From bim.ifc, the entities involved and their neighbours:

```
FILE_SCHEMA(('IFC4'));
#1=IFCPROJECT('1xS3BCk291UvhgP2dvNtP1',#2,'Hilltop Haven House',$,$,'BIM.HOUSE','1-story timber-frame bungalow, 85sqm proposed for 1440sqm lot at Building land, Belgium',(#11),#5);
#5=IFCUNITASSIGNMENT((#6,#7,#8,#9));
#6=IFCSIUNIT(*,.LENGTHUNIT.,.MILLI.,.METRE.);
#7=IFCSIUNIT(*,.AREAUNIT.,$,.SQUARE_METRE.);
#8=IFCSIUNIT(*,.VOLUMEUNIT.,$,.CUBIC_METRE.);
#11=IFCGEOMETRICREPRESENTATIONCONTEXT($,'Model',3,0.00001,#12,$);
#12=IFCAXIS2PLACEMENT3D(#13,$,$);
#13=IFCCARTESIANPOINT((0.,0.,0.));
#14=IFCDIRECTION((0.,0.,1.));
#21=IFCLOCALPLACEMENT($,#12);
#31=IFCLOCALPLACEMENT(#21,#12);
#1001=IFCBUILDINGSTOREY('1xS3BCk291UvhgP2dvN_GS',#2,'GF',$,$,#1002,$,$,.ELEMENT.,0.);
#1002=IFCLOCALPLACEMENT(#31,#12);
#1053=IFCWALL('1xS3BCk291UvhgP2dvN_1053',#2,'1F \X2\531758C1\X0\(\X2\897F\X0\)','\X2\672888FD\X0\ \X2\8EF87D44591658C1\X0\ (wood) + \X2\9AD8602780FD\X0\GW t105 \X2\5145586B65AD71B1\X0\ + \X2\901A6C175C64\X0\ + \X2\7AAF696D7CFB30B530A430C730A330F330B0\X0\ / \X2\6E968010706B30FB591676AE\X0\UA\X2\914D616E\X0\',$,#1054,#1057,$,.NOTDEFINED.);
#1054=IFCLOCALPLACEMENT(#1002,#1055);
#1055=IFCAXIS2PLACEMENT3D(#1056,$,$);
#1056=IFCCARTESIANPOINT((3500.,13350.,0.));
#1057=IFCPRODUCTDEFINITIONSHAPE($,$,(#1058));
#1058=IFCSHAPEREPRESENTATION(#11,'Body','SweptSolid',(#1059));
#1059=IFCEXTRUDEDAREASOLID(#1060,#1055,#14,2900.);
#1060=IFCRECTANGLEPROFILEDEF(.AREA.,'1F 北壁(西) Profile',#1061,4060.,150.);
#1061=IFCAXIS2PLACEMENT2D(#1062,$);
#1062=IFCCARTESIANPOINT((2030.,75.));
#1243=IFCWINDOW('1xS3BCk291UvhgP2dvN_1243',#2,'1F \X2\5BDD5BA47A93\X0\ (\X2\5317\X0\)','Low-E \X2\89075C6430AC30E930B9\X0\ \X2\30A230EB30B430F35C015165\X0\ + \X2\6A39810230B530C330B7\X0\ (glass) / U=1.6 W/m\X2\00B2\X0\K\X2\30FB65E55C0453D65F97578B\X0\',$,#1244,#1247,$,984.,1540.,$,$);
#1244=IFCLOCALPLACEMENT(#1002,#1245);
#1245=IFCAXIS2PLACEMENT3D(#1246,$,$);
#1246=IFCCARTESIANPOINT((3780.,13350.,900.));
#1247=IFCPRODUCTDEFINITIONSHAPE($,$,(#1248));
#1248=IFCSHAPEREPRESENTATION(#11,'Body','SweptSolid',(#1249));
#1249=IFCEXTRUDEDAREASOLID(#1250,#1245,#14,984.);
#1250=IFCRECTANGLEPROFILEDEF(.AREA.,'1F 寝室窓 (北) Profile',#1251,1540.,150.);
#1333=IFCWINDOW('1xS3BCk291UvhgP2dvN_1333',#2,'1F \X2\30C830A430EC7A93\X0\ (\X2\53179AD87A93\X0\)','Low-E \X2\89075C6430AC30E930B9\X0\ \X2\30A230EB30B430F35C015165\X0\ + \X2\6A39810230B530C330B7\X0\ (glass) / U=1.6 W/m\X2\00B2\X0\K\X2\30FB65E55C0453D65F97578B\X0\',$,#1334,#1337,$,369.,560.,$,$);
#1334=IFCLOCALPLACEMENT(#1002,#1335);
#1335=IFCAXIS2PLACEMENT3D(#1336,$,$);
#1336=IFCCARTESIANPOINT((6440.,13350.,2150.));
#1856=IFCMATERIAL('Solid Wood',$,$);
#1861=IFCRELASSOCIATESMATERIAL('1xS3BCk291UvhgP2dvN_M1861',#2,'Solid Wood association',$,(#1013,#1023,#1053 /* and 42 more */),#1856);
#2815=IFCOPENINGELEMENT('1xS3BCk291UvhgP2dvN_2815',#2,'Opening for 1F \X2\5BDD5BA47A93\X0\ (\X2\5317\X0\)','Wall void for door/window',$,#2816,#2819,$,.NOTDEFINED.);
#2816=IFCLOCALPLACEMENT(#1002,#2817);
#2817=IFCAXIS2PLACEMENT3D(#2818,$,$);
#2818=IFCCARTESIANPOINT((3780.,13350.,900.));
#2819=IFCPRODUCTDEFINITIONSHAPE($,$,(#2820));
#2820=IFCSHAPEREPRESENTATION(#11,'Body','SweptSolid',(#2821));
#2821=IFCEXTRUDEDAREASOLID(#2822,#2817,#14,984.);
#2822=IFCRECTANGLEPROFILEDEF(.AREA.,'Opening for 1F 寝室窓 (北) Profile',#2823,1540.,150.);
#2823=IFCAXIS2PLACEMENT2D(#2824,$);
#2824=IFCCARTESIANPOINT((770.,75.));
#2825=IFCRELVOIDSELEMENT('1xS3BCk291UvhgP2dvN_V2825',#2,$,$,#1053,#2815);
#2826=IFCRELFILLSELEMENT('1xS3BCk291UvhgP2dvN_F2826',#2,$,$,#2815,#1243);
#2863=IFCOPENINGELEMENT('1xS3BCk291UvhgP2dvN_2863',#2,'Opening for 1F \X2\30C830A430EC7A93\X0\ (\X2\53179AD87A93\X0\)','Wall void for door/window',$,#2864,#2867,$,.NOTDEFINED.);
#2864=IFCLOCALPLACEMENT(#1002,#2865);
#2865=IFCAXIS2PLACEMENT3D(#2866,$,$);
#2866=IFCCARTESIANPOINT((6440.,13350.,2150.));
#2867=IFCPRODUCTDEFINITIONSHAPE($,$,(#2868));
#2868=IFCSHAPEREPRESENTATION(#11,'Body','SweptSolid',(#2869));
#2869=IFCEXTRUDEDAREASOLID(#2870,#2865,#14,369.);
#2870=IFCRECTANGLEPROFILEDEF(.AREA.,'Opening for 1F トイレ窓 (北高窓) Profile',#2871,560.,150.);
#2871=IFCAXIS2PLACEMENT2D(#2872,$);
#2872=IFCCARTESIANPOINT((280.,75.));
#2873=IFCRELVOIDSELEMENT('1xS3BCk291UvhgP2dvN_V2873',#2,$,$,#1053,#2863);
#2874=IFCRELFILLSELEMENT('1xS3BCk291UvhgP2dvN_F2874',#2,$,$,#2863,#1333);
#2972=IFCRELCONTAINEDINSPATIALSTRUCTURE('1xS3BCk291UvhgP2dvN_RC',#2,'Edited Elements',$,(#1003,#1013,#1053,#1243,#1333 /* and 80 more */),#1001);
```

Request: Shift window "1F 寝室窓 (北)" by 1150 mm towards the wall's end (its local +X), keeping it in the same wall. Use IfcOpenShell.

```python
import ifcopenshell
import ifcopenshell.api.geometry
import ifcopenshell.util.placement
import ifcopenshell.util.unit

model = ifcopenshell.open("bim.ifc")
unit_scale = ifcopenshell.util.unit.calculate_unit_scale(model)

window = model.by_guid("1xS3BCk291UvhgP2dvN_1243")
opening = window.FillsVoids[0].RelatingOpeningElement
wall = opening.VoidsElements[0].RelatingBuildingElement

wall_matrix = ifcopenshell.util.placement.get_local_placement(wall.ObjectPlacement)
shift = wall_matrix[:3, 0] * 1.15 / unit_scale
before = ifcopenshell.util.placement.get_local_placement(window.ObjectPlacement)[:3, 3].copy()

# The window is not placed relative to its opening, so move both.
for product in (opening, window):
    matrix = ifcopenshell.util.placement.get_local_placement(product.ObjectPlacement)
    matrix[:3, 3] += shift
    ifcopenshell.api.geometry.edit_object_placement(model, product=product, matrix=matrix, is_si=False)

after = ifcopenshell.util.placement.get_local_placement(window.ObjectPlacement)[:3, 3]
print("window moved by", (after - before).round(3) + 0.0)

model.write("bim_v2.ifc")
```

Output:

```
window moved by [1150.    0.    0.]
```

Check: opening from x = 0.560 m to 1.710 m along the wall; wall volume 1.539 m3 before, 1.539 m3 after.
